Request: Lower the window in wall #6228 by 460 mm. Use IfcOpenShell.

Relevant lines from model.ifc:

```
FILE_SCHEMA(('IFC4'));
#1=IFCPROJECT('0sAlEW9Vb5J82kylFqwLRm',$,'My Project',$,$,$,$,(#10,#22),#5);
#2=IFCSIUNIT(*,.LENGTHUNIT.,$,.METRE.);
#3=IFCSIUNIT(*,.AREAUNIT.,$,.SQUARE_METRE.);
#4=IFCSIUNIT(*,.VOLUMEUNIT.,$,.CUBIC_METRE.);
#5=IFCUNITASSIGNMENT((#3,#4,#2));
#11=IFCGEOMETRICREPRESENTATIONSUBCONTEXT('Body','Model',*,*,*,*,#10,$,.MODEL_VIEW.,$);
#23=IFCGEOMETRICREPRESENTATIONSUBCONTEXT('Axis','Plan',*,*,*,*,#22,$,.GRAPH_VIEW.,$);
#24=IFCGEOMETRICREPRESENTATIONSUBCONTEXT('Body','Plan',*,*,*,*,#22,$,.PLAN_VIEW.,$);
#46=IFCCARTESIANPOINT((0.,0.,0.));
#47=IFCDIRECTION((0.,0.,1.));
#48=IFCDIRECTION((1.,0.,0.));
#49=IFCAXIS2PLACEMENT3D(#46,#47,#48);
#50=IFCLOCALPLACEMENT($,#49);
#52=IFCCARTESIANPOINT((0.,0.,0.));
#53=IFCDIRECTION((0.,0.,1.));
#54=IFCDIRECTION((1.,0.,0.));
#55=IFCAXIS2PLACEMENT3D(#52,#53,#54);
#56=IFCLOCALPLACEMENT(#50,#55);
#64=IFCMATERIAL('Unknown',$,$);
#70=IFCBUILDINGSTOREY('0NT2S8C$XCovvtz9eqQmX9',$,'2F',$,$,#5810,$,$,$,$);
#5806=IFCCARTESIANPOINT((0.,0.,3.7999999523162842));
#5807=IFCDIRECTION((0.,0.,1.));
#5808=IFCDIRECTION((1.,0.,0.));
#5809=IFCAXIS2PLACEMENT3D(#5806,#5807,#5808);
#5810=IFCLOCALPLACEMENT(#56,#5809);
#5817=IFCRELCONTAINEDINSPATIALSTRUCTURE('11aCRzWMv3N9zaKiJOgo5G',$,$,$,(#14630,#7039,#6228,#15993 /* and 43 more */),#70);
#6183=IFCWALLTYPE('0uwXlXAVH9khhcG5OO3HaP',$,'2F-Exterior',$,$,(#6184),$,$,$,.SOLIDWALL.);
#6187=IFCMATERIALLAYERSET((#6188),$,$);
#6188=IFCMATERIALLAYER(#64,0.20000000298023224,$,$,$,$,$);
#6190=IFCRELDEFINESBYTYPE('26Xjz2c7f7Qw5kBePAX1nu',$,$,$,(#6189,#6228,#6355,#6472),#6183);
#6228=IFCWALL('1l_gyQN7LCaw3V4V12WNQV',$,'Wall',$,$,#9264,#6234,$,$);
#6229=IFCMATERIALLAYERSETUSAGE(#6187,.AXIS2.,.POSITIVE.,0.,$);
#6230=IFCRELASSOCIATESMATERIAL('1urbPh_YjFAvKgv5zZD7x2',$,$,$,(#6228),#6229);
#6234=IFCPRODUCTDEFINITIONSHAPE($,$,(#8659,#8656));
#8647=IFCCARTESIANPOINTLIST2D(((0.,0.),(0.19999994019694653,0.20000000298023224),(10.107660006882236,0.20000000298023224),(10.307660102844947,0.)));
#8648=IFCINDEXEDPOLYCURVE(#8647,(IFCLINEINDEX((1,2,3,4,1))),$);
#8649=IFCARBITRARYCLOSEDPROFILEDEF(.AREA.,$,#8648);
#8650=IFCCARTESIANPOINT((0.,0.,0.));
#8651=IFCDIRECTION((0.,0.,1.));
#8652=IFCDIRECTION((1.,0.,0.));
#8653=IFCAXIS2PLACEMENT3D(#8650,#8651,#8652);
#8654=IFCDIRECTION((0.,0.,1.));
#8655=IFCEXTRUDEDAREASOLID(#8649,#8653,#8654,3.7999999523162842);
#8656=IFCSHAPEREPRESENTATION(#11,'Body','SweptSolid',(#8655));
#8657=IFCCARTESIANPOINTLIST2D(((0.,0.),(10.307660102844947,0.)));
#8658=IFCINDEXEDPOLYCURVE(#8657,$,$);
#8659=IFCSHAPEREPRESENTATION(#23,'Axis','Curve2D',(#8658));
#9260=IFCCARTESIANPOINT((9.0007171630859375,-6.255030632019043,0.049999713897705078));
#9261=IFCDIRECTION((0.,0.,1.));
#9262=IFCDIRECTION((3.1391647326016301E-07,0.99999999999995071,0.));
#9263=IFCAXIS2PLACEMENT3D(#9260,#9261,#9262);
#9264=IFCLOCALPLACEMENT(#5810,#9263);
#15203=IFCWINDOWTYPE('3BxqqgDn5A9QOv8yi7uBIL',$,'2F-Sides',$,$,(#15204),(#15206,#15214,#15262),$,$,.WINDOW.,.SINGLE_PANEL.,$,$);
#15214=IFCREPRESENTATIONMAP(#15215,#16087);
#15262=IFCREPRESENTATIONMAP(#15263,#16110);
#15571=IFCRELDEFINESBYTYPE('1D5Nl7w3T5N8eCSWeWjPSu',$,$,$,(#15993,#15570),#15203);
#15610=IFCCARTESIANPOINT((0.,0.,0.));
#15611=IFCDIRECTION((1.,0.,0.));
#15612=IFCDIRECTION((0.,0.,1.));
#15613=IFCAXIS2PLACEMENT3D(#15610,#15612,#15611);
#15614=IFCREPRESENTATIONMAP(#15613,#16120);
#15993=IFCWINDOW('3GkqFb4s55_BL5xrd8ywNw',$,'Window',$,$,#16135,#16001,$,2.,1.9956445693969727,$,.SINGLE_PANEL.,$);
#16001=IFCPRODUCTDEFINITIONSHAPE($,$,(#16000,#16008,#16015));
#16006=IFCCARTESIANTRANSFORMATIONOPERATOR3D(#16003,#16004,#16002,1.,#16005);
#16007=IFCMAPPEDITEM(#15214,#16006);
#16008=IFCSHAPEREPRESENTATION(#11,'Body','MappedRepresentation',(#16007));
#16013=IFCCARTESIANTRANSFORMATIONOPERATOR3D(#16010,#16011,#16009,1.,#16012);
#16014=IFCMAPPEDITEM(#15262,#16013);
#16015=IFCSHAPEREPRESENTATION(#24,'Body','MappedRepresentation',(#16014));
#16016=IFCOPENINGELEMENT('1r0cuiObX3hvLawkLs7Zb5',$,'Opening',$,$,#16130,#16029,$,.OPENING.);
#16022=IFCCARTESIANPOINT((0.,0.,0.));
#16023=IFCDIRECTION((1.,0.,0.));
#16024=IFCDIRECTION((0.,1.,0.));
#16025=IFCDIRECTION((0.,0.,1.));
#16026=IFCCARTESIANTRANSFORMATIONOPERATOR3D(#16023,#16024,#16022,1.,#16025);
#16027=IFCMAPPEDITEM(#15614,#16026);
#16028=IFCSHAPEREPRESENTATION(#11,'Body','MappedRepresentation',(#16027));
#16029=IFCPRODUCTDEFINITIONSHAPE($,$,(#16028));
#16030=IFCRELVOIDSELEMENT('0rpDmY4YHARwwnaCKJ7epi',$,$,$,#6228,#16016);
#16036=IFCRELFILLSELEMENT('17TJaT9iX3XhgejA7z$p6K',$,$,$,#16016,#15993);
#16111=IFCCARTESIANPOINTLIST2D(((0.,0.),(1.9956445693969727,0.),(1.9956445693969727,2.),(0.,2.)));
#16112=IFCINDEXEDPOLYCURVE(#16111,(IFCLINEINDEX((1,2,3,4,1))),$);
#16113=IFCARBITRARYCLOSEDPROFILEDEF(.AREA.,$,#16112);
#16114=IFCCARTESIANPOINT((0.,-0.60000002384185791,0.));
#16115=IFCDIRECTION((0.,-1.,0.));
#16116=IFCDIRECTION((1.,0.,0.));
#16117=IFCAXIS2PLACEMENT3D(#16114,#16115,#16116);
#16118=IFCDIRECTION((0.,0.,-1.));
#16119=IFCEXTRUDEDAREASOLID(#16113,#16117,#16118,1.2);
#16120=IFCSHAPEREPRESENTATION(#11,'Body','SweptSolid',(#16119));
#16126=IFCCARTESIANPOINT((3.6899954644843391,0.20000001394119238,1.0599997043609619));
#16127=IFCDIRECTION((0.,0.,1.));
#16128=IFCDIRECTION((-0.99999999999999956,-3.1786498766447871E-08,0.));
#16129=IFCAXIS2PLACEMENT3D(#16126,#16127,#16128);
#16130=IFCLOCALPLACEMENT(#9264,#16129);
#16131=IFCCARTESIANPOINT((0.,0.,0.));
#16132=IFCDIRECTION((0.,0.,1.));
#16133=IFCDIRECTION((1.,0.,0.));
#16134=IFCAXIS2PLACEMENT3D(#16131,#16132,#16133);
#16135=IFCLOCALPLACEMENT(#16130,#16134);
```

```python
import numpy as np
import ifcopenshell
import ifcopenshell.api.geometry
import ifcopenshell.util.placement
import ifcopenshell.util.unit

model = ifcopenshell.open("model.ifc")
unit_scale = ifcopenshell.util.unit.calculate_unit_scale(model)

window = model.by_id(15993)
opening = window.FillsVoids[0].RelatingOpeningElement
dz = -0.46

shift = np.array([0.0, 0.0, dz])
# The window is placed relative to its opening, so it follows when the opening moves.
matrix = ifcopenshell.util.placement.get_local_placement(opening.ObjectPlacement)
matrix[:3, 3] += shift
ifcopenshell.api.geometry.edit_object_placement(
    model, product=opening, matrix=matrix, is_si=False, should_transform_children=True
)

print(f"moved by {dz * unit_scale:+.3f} m")

model.write("model_rev.ifc")
```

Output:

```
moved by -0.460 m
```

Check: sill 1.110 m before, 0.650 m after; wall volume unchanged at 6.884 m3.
